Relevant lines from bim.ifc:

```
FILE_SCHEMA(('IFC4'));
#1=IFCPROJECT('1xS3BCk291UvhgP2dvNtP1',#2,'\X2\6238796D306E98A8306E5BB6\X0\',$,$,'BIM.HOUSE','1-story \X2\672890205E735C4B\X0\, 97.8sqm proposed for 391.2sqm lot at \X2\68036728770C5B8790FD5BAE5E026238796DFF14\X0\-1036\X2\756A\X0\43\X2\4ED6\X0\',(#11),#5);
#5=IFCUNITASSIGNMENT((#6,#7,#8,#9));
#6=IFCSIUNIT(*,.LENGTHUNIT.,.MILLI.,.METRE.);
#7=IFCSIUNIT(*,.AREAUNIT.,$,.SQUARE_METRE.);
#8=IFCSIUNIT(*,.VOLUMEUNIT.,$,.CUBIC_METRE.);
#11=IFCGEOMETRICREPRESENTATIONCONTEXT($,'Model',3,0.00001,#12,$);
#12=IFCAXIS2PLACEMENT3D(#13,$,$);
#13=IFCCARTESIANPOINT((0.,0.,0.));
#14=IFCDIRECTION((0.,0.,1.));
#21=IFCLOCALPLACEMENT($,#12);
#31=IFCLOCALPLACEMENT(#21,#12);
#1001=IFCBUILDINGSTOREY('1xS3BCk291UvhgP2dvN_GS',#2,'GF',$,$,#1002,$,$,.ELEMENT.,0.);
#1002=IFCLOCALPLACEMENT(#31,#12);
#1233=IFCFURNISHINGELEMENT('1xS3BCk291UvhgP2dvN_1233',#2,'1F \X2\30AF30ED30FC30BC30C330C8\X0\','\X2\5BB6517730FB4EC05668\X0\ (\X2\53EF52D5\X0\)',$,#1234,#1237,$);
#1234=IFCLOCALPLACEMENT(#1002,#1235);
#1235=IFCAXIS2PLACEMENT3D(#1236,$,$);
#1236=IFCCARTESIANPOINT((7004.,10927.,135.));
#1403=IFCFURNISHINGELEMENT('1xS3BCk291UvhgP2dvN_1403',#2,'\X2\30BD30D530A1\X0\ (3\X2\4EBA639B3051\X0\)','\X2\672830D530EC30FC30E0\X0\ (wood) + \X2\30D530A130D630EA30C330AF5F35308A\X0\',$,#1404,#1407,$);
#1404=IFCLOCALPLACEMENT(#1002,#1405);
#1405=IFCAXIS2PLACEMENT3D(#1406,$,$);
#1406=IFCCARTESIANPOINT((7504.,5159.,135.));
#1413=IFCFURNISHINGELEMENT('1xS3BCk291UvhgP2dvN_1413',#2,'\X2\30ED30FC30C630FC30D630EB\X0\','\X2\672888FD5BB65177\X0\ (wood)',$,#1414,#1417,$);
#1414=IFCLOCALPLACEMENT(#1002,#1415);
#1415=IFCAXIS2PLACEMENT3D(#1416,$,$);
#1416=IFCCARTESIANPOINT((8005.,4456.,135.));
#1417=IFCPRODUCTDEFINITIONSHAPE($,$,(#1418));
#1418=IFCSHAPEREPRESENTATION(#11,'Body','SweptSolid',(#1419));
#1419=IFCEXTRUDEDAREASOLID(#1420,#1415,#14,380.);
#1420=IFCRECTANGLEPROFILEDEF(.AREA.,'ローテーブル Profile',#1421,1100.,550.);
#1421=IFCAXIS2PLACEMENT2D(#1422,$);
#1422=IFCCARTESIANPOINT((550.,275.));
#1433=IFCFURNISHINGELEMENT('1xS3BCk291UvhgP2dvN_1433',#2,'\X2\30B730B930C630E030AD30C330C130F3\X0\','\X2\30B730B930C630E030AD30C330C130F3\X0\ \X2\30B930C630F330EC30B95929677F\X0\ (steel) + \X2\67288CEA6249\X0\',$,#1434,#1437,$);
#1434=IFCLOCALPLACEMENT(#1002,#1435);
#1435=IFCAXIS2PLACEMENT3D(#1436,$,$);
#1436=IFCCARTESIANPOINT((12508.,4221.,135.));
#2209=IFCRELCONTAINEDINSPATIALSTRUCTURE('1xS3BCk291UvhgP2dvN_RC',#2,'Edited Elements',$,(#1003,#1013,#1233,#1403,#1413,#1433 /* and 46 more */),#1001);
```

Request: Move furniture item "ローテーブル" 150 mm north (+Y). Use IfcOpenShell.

```python
import ifcopenshell
import ifcopenshell.api.geometry
import ifcopenshell.util.placement
import ifcopenshell.util.unit

model = ifcopenshell.open("bim.ifc")
unit_scale = ifcopenshell.util.unit.calculate_unit_scale(model)

item = model.by_guid("1xS3BCk291UvhgP2dvN_1413")
matrix = ifcopenshell.util.placement.get_local_placement(item.ObjectPlacement)
matrix[1, 3] += 0.15 / unit_scale
ifcopenshell.api.geometry.edit_object_placement(model, product=item, matrix=matrix, is_si=False)

print(ifcopenshell.util.placement.get_local_placement(item.ObjectPlacement).round(3) + 0.0)

model.write("bim_v2.ifc")
```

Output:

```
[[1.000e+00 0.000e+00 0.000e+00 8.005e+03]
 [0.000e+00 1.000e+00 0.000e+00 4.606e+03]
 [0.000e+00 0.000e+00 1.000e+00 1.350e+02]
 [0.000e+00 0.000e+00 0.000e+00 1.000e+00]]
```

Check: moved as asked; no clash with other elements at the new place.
